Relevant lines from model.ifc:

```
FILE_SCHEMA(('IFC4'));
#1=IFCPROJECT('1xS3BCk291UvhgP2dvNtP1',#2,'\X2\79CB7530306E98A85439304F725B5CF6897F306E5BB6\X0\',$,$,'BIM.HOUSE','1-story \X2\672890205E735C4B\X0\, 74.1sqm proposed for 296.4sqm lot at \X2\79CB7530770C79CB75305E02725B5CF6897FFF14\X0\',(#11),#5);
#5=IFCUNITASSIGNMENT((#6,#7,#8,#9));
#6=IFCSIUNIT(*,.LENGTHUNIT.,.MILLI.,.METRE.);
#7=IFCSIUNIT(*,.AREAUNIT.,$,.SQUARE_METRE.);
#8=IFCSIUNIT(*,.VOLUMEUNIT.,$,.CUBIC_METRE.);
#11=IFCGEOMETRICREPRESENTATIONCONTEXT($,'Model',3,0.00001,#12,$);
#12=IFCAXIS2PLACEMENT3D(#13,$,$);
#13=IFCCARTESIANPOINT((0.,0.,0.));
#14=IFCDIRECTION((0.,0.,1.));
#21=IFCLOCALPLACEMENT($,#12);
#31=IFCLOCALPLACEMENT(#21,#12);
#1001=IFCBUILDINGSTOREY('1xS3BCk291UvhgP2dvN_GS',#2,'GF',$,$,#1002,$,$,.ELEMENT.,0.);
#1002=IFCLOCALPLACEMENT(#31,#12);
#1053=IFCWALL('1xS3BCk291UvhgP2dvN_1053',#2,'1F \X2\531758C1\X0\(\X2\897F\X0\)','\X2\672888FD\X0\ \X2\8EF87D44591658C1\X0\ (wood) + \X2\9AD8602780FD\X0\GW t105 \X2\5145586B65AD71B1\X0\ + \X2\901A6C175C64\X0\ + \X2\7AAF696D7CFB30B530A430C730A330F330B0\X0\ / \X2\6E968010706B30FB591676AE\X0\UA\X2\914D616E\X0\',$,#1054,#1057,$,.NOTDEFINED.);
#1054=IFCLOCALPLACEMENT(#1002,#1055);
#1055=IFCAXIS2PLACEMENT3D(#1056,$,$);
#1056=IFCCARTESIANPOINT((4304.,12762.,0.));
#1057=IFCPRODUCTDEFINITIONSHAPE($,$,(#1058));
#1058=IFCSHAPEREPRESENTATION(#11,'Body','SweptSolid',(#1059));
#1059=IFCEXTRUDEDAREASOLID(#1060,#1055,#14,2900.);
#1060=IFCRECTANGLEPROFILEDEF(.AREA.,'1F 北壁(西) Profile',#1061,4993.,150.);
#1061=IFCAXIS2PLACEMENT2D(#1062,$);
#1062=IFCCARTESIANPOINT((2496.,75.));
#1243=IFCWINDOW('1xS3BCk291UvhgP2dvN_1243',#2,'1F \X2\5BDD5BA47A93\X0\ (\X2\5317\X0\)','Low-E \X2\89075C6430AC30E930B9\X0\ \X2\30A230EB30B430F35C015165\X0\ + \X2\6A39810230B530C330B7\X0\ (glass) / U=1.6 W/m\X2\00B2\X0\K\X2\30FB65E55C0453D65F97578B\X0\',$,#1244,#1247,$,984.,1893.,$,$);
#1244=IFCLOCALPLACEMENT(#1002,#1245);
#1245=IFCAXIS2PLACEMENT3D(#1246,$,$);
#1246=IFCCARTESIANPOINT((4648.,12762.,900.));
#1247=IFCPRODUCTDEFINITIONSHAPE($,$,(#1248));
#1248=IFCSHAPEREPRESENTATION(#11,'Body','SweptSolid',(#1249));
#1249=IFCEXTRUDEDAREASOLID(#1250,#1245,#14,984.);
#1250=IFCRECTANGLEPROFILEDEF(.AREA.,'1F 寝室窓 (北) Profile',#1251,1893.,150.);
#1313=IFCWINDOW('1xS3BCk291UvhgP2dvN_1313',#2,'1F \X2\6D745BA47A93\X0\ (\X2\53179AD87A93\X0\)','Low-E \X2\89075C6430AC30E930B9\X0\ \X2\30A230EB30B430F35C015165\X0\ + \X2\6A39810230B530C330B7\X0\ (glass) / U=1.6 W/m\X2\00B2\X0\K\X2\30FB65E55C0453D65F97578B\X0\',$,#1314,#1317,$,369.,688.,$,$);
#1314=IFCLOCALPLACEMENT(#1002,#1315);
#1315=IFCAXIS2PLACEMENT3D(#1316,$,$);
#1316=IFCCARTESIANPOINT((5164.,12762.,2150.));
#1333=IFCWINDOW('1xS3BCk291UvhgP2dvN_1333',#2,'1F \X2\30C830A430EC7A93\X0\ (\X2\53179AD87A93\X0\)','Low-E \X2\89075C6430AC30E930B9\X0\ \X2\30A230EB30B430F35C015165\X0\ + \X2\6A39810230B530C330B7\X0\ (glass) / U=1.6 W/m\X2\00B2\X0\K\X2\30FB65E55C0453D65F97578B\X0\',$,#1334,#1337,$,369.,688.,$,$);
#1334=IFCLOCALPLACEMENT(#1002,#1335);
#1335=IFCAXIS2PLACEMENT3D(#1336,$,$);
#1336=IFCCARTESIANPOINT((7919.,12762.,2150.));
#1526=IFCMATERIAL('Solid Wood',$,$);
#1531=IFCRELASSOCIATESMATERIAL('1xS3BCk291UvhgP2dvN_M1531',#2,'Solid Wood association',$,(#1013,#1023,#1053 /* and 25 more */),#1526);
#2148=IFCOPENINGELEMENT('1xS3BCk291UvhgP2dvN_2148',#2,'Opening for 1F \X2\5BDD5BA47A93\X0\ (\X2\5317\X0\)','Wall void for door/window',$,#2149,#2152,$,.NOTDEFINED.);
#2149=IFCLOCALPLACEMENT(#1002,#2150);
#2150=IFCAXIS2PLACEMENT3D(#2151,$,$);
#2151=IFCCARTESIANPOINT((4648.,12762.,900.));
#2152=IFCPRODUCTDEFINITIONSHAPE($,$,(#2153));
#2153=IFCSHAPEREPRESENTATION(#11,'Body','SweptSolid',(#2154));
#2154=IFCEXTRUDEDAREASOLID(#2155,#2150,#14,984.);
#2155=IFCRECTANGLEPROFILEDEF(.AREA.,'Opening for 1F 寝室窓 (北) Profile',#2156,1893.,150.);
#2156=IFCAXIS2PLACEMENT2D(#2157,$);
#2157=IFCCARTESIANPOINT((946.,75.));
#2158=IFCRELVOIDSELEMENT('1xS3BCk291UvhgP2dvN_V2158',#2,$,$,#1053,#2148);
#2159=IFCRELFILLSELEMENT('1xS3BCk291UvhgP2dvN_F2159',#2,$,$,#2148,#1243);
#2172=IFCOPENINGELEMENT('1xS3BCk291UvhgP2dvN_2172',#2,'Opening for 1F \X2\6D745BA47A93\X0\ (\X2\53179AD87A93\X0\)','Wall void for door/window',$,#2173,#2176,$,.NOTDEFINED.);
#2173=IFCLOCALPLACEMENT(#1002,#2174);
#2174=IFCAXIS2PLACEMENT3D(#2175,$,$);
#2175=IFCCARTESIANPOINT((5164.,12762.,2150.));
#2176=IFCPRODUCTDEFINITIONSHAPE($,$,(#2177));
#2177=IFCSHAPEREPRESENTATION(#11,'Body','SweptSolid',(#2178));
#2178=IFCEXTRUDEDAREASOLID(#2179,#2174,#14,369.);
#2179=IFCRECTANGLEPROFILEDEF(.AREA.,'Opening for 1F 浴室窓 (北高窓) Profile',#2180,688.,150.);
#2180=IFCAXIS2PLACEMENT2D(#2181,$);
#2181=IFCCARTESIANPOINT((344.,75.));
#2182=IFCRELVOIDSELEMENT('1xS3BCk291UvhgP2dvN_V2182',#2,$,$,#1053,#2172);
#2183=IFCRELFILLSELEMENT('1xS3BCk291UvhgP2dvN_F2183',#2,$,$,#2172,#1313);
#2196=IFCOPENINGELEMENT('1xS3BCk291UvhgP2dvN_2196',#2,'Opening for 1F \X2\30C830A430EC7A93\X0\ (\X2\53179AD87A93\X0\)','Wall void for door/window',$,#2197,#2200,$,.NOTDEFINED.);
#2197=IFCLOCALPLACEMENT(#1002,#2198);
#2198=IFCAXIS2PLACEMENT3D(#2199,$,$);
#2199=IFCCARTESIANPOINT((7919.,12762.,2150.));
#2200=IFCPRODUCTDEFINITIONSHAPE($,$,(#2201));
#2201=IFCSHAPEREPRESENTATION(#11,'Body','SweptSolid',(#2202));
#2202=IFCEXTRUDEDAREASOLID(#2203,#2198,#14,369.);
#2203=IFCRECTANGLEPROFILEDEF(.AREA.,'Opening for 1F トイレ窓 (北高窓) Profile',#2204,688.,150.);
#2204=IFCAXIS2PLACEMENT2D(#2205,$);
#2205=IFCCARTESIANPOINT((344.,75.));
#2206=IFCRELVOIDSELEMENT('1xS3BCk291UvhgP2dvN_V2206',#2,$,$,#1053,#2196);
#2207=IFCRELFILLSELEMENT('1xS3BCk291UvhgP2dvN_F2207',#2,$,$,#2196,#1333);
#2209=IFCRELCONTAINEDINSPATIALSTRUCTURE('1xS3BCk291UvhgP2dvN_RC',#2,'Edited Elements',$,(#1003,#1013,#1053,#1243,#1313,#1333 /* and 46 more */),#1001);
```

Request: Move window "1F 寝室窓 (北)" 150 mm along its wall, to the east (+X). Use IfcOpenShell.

```python
import ifcopenshell
import ifcopenshell.api.geometry
import ifcopenshell.util.placement
import ifcopenshell.util.unit

model = ifcopenshell.open("model.ifc")
unit_scale = ifcopenshell.util.unit.calculate_unit_scale(model)

window = model.by_guid("1xS3BCk291UvhgP2dvN_1243")
opening = window.FillsVoids[0].RelatingOpeningElement
wall = opening.VoidsElements[0].RelatingBuildingElement

wall_matrix = ifcopenshell.util.placement.get_local_placement(wall.ObjectPlacement)
shift = wall_matrix[:3, 0] * 0.15 / unit_scale
before = ifcopenshell.util.placement.get_local_placement(window.ObjectPlacement)[:3, 3].copy()

# The window is not placed relative to its opening, so move both.
for product in (opening, window):
    matrix = ifcopenshell.util.placement.get_local_placement(product.ObjectPlacement)
    matrix[:3, 3] += shift
    ifcopenshell.api.geometry.edit_object_placement(model, product=product, matrix=matrix, is_si=False)

after = ifcopenshell.util.placement.get_local_placement(window.ObjectPlacement)[:3, 3]
print("window moved by", (after - before).round(3) + 0.0)

model.write("model_updated.ifc")
```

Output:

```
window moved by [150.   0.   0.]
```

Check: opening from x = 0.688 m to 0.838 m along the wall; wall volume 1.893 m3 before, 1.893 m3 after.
